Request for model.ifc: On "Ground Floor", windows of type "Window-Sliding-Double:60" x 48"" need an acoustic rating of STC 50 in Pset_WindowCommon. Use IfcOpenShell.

First a look at what the model holds.

```python
import ifcopenshell
import ifcopenshell.util.element

model = ifcopenshell.open("model.ifc")
print(model.schema)
storey = next(s for s in model.by_type("IfcBuildingStorey") if s.Name == "Ground Floor")
windows = [e for e in ifcopenshell.util.element.get_decomposition(storey) if e.is_a("IfcWindow")]
seen = {}
for e in windows:
    element_type = ifcopenshell.util.element.get_type(e)
    key = (element_type.Name if element_type != e and element_type else None, ifcopenshell.util.element.get_pset(e, "Pset_WindowCommon", "AcousticRating"))
    seen[key] = seen.get(key, 0) + 1
for (name, value), count in sorted(seen.items(), key=str):
    print(count, "x", name, "|", value)
```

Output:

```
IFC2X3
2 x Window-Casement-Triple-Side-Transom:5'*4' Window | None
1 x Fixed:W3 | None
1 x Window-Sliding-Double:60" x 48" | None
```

```python
import ifcopenshell
import ifcopenshell.api.pset
import ifcopenshell.util.element

model = ifcopenshell.open("model.ifc")

storey = next(s for s in model.by_type("IfcBuildingStorey") if s.Name == "Ground Floor")
windows = [e for e in ifcopenshell.util.element.get_decomposition(storey) if e.is_a("IfcWindow")]

count = 0
for e in windows:
    element_type = ifcopenshell.util.element.get_type(e)
    if element_type in (None, e) or element_type.Name != 'Window-Sliding-Double:60" x 48"':
        continue
    # add_pset returns the element's existing set when there is one.
    pset = ifcopenshell.api.pset.add_pset(model, product=e, name="Pset_WindowCommon")
    ifcopenshell.api.pset.edit_pset(model, pset=pset, properties={"AcousticRating": "STC 50"})
    count += 1

print(count, "windows updated")

model.write("model_updated.ifc")
```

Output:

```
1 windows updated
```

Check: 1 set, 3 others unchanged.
